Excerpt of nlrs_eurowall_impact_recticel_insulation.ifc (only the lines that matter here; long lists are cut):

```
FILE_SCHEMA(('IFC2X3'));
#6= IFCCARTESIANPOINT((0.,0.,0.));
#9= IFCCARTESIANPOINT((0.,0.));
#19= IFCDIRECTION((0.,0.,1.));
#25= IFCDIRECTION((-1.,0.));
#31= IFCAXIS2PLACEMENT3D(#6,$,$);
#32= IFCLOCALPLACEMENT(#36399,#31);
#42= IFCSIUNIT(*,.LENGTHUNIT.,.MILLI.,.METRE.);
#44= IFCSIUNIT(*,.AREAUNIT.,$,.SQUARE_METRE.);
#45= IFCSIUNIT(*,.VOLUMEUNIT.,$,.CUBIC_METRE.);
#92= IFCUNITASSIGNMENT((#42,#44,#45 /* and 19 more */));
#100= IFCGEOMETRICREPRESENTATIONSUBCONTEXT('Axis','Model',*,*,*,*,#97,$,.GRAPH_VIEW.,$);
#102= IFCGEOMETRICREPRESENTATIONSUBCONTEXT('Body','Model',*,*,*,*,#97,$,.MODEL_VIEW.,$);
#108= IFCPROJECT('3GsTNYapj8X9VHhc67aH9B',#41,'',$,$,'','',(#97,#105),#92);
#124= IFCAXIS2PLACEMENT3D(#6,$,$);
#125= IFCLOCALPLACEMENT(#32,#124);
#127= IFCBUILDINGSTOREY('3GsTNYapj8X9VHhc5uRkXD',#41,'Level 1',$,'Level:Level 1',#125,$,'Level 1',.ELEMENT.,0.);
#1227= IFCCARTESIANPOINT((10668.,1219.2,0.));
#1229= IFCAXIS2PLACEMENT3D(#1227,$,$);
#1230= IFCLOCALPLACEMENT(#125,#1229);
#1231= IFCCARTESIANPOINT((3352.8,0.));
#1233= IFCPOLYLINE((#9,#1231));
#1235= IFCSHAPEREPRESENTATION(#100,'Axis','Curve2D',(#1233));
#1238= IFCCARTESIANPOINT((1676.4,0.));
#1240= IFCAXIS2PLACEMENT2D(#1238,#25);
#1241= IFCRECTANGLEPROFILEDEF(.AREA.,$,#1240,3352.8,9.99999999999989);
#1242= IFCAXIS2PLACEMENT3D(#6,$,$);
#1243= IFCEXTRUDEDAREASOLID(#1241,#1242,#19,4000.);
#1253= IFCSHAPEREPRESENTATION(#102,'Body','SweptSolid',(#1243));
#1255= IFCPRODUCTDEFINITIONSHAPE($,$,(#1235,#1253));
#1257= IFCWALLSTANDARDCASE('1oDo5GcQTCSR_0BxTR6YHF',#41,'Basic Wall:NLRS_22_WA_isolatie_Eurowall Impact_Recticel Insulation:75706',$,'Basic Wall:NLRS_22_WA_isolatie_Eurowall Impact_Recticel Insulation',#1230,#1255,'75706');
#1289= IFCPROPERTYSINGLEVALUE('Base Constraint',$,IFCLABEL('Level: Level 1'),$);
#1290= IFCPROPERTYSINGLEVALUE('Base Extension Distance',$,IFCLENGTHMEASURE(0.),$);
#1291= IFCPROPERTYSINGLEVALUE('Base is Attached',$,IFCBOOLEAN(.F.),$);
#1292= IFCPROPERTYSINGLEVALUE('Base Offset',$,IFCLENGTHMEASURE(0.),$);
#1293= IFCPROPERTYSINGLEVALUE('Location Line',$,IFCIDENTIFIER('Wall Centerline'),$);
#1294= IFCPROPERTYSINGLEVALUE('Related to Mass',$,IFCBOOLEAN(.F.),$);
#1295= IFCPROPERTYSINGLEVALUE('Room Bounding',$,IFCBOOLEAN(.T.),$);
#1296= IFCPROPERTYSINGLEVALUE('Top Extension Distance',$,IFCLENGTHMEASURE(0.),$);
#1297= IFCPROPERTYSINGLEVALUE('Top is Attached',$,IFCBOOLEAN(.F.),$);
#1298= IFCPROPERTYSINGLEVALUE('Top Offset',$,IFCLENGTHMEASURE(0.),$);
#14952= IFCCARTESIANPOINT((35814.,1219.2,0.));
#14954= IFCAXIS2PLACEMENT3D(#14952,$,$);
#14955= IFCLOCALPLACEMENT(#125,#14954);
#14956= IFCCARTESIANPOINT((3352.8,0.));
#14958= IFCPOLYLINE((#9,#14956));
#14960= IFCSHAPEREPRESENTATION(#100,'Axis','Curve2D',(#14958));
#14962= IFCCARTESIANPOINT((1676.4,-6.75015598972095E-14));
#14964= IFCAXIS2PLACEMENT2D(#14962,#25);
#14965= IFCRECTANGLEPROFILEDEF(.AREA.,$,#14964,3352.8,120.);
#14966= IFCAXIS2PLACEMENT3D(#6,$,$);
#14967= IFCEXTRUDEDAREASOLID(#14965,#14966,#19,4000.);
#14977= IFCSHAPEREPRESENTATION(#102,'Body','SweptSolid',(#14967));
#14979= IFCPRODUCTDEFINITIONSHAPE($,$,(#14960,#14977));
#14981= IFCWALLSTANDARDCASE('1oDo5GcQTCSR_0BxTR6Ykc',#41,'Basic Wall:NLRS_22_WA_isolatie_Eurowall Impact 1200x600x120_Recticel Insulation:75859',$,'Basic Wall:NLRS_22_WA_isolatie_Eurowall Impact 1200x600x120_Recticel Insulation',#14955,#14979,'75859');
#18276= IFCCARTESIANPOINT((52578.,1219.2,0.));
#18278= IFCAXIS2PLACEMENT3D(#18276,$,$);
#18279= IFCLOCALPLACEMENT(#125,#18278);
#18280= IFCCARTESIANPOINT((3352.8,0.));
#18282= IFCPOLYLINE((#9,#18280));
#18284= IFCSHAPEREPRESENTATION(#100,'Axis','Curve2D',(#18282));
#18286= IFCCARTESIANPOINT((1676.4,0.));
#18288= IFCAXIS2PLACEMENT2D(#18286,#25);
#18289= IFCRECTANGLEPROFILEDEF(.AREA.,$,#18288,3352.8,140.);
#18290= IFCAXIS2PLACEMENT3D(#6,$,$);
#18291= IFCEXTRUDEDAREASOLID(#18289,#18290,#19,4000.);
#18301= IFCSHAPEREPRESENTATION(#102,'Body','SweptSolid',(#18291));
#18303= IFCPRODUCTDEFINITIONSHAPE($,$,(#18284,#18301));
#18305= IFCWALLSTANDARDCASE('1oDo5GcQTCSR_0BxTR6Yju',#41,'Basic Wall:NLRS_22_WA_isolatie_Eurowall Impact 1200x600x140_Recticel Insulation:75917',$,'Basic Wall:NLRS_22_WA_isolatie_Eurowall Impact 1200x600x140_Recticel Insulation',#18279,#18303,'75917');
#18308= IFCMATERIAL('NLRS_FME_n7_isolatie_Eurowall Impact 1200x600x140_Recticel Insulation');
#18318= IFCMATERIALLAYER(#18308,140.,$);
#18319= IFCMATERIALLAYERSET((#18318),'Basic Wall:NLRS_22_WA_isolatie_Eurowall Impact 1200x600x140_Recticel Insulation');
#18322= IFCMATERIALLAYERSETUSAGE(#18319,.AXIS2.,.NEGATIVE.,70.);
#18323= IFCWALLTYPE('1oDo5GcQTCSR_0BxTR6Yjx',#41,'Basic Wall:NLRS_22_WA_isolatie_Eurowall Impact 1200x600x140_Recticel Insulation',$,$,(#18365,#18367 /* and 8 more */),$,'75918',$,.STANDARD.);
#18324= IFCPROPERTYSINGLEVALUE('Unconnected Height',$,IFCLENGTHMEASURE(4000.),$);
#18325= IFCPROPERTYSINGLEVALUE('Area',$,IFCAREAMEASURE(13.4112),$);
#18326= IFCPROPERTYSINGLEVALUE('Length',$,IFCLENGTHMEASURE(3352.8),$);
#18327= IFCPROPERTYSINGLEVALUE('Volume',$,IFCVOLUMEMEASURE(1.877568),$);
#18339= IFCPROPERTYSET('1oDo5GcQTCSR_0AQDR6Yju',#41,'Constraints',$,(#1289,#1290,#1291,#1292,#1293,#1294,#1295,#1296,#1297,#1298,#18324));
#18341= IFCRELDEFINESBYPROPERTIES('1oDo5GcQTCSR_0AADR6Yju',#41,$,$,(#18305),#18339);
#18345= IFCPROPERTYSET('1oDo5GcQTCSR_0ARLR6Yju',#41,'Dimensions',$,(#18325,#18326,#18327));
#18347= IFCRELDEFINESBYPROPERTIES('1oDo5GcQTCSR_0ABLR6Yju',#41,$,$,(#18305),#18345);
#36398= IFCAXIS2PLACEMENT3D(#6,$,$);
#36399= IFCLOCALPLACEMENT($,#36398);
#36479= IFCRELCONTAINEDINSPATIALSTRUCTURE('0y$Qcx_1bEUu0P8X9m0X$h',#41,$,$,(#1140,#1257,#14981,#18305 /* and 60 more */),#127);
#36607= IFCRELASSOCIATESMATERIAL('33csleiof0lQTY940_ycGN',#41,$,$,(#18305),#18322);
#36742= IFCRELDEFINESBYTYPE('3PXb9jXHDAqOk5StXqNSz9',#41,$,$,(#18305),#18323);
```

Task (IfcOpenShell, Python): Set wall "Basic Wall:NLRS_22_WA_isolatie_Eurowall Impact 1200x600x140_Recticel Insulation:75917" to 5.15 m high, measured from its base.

```python
import ifcopenshell
import ifcopenshell.api.pset
import ifcopenshell.geom
import ifcopenshell.util.element
import ifcopenshell.util.representation
import ifcopenshell.util.shape
import ifcopenshell.util.unit

model = ifcopenshell.open("nlrs_eurowall_impact_recticel_insulation.ifc")
unit_scale = ifcopenshell.util.unit.calculate_unit_scale(model)
area_scale = ifcopenshell.util.unit.calculate_unit_scale(model, "AREAUNIT")
volume_scale = ifcopenshell.util.unit.calculate_unit_scale(model, "VOLUMEUNIT")
settings = ifcopenshell.geom.settings()


def volume(element):
    """Net volume in cubic metres, openings subtracted."""
    shape = ifcopenshell.geom.create_shape(settings, element)
    return ifcopenshell.util.shape.get_volume(shape.geometry)


wall = model.by_guid("1oDo5GcQTCSR_0BxTR6Yju")
before = volume(wall)

body = ifcopenshell.util.representation.get_representation(wall, "Model", "Body")
solid = body.Items[0]
old_height = solid.Depth
solid.Depth = 5.15 / unit_scale
after = volume(wall)
thickness = 0.14  # wall thickness in metres

# Update the stored height, areas and volumes.
pset = model.by_id(ifcopenshell.util.element.get_pset(wall, "Constraints", should_inherit=False)["id"])
ifcopenshell.api.pset.edit_pset(model, pset=pset, properties={
    "Unconnected Height": model.create_entity("IfcLengthMeasure", solid.Depth),
})
pset = model.by_id(ifcopenshell.util.element.get_pset(wall, "Dimensions", should_inherit=False)["id"])
ifcopenshell.api.pset.edit_pset(model, pset=pset, properties={
    "Area": model.create_entity("IfcAreaMeasure", after / thickness / area_scale),
    "Volume": model.create_entity("IfcVolumeMeasure", after / volume_scale),
})

print(f"height {old_height:g} -> {solid.Depth:g}, volume {before:.3f} -> {after:.3f} m3")

model.write("nlrs_eurowall_impact_recticel_insulation_v2.ifc")
```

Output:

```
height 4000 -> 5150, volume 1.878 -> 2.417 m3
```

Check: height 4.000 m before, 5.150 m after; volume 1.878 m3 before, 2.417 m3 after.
